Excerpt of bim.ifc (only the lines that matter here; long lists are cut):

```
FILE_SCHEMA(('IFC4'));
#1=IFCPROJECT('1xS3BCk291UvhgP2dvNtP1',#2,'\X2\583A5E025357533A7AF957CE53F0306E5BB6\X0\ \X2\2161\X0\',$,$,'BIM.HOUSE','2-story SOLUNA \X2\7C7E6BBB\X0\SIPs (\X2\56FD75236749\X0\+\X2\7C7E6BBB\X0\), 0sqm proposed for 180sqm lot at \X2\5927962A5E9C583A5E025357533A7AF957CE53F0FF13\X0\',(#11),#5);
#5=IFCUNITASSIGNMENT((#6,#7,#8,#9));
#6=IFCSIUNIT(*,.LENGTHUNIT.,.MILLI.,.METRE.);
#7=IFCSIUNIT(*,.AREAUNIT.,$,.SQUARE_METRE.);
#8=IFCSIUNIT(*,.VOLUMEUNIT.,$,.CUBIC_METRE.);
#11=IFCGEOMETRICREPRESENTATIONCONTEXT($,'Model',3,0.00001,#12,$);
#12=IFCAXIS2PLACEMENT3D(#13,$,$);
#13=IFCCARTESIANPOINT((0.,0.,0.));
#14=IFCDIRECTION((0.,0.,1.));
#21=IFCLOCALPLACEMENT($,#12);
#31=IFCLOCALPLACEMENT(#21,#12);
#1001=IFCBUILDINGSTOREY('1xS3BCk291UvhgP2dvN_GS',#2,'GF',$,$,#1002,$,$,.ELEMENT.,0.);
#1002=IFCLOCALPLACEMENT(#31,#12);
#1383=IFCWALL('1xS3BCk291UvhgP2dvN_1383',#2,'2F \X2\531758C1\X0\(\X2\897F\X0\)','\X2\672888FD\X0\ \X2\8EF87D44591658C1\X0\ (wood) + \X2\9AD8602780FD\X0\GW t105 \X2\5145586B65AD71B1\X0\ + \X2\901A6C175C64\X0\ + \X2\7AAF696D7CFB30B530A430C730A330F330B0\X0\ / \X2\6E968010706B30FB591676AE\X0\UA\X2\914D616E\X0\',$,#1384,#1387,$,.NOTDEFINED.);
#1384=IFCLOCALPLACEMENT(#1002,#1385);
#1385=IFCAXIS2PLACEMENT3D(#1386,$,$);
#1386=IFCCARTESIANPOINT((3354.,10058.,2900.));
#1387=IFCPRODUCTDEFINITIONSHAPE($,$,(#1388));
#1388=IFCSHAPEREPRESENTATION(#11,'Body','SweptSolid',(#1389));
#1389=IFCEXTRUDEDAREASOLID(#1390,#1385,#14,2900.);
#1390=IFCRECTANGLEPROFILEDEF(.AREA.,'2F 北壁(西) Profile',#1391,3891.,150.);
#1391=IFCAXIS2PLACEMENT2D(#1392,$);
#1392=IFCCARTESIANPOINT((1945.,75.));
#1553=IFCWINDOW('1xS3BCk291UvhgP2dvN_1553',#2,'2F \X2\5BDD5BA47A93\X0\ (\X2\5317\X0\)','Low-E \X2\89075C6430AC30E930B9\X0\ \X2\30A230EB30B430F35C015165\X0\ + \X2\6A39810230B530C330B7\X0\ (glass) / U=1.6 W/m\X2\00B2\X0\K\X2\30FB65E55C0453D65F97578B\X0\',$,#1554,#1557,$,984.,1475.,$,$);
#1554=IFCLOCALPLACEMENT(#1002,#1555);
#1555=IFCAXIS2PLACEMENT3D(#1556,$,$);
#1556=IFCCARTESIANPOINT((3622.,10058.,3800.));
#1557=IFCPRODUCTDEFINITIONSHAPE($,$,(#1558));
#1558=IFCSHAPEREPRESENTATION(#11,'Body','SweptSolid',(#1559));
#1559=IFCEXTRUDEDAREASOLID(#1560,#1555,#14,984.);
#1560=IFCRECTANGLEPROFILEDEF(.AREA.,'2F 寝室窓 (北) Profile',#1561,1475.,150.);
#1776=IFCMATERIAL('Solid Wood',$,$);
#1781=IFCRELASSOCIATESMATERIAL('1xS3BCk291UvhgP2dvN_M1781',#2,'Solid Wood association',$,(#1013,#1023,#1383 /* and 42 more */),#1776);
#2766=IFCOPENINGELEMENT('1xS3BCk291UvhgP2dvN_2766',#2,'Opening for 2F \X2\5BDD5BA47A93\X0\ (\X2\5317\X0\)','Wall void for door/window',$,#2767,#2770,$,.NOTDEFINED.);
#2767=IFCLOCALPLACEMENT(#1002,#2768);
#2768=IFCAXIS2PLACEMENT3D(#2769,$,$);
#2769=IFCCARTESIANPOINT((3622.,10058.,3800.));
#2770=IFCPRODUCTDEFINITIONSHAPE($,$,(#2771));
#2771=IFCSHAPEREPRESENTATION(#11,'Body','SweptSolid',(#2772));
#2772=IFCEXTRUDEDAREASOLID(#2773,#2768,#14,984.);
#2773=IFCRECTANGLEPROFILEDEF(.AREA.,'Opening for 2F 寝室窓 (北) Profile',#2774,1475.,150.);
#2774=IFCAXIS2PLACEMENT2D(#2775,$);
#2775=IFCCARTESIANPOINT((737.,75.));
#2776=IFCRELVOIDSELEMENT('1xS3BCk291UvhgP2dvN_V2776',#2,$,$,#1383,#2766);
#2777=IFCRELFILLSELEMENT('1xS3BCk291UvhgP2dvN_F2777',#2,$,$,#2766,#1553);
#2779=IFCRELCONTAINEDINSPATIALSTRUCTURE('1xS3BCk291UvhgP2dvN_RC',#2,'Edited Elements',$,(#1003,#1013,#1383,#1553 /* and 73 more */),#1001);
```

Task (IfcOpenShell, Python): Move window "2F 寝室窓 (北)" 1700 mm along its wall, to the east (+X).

```python
import ifcopenshell
import ifcopenshell.api.geometry
import ifcopenshell.util.placement
import ifcopenshell.util.unit

model = ifcopenshell.open("bim.ifc")
unit_scale = ifcopenshell.util.unit.calculate_unit_scale(model)

window = model.by_guid("1xS3BCk291UvhgP2dvN_1553")
opening = window.FillsVoids[0].RelatingOpeningElement
wall = opening.VoidsElements[0].RelatingBuildingElement

wall_matrix = ifcopenshell.util.placement.get_local_placement(wall.ObjectPlacement)
shift = wall_matrix[:3, 0] * 1.7 / unit_scale
before = ifcopenshell.util.placement.get_local_placement(window.ObjectPlacement)[:3, 3].copy()

# The window is not placed relative to its opening, so move both.
for product in (opening, window):
    matrix = ifcopenshell.util.placement.get_local_placement(product.ObjectPlacement)
    matrix[:3, 3] += shift
    ifcopenshell.api.geometry.edit_object_placement(model, product=product, matrix=matrix, is_si=False)

after = ifcopenshell.util.placement.get_local_placement(window.ObjectPlacement)[:3, 3]
print("window moved by", (after - before).round(3) + 0.0)

model.write("bim_edited.ifc")
```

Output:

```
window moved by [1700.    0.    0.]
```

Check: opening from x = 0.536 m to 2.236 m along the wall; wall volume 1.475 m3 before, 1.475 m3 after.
